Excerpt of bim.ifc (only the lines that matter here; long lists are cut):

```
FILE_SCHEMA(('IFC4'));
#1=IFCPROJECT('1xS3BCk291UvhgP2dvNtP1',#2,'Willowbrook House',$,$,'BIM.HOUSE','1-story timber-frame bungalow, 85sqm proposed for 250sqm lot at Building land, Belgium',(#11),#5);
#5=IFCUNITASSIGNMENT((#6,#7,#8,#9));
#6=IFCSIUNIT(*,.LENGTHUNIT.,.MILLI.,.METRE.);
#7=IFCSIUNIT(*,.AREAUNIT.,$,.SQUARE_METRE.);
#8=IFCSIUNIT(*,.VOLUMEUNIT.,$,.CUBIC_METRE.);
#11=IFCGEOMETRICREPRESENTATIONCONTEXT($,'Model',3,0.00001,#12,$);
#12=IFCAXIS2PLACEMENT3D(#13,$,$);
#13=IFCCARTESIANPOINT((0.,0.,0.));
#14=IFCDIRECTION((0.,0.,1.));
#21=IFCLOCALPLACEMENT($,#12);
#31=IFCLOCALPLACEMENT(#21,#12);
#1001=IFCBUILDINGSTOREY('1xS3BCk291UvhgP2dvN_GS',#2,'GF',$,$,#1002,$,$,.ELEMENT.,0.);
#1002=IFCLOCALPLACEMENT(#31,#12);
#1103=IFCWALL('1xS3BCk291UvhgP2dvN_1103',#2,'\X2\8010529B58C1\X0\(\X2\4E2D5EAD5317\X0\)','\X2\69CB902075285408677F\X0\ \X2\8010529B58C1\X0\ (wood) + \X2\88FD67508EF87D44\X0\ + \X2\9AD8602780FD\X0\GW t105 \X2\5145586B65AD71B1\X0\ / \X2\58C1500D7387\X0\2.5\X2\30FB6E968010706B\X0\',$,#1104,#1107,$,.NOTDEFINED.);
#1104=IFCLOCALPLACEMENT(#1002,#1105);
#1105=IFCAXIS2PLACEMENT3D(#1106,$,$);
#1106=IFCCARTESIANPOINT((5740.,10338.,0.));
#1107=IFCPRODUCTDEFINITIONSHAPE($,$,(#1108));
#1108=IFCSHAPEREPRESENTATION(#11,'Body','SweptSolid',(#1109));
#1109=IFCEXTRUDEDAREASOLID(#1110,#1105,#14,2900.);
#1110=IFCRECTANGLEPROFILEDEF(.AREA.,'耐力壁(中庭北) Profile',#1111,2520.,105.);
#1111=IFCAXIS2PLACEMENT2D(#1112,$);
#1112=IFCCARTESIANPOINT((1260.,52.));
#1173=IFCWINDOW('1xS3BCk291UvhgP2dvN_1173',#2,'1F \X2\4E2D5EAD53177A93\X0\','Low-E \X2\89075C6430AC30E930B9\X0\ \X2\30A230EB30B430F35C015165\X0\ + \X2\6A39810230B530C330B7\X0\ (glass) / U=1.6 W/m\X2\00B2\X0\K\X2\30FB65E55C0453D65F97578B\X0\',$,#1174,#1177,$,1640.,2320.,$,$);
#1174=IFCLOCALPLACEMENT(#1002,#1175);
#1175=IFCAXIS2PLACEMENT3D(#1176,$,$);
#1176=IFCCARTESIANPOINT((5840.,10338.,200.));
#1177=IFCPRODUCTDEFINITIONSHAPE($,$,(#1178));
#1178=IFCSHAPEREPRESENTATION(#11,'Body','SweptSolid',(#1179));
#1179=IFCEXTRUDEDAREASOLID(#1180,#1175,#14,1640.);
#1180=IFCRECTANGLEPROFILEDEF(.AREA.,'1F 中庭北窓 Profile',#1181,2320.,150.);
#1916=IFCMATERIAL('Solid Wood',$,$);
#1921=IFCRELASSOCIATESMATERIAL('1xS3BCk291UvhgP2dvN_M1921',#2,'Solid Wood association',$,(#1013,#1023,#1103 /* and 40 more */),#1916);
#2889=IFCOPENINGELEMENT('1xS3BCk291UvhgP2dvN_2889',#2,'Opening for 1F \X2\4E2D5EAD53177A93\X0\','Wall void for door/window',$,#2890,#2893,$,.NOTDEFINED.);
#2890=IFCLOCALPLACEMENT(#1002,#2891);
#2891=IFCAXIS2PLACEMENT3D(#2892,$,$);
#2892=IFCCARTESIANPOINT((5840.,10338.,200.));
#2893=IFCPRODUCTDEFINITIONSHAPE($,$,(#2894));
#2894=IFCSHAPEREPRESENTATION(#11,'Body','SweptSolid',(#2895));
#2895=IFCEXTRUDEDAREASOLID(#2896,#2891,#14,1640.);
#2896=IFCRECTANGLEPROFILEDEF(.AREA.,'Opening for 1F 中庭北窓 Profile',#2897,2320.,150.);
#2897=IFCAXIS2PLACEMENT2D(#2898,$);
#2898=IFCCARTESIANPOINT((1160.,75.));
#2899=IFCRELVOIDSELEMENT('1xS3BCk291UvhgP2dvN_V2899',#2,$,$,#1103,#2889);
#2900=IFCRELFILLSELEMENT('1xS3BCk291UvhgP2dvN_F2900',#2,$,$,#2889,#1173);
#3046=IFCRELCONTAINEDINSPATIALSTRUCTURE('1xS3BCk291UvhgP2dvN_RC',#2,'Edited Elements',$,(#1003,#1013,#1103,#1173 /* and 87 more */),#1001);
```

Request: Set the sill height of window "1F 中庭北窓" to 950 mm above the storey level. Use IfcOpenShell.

```python
import numpy as np
import ifcopenshell
import ifcopenshell.api.geometry
import ifcopenshell.geom
import ifcopenshell.util.element
import ifcopenshell.util.placement
import ifcopenshell.util.shape
import ifcopenshell.util.unit

model = ifcopenshell.open("bim.ifc")
unit_scale = ifcopenshell.util.unit.calculate_unit_scale(model)

window = model.by_guid("1xS3BCk291UvhgP2dvN_1173")
opening = window.FillsVoids[0].RelatingOpeningElement
storey = ifcopenshell.util.element.get_container(window, ifc_class="IfcBuildingStorey")
level = ifcopenshell.util.placement.get_local_placement(storey.ObjectPlacement)[2, 3]

# The opening's origin need not be at the sill, so measure its lowest point.
shape = ifcopenshell.geom.create_shape(ifcopenshell.geom.settings(), opening)
bottom = ifcopenshell.util.shape.get_shape_bottom_elevation(shape, shape.geometry) / unit_scale
dz = level + 950.0 - bottom

shift = np.array([0.0, 0.0, dz])
# The window is not placed relative to its opening, so move both.
for product in (opening, window):
    matrix = ifcopenshell.util.placement.get_local_placement(product.ObjectPlacement)
    matrix[:3, 3] += shift
    ifcopenshell.api.geometry.edit_object_placement(model, product=product, matrix=matrix, is_si=False)

print(f"moved by {dz * unit_scale:+.3f} m")

model.write("bim_v2.ifc")
```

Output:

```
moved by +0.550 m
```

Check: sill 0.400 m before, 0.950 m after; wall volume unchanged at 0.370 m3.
